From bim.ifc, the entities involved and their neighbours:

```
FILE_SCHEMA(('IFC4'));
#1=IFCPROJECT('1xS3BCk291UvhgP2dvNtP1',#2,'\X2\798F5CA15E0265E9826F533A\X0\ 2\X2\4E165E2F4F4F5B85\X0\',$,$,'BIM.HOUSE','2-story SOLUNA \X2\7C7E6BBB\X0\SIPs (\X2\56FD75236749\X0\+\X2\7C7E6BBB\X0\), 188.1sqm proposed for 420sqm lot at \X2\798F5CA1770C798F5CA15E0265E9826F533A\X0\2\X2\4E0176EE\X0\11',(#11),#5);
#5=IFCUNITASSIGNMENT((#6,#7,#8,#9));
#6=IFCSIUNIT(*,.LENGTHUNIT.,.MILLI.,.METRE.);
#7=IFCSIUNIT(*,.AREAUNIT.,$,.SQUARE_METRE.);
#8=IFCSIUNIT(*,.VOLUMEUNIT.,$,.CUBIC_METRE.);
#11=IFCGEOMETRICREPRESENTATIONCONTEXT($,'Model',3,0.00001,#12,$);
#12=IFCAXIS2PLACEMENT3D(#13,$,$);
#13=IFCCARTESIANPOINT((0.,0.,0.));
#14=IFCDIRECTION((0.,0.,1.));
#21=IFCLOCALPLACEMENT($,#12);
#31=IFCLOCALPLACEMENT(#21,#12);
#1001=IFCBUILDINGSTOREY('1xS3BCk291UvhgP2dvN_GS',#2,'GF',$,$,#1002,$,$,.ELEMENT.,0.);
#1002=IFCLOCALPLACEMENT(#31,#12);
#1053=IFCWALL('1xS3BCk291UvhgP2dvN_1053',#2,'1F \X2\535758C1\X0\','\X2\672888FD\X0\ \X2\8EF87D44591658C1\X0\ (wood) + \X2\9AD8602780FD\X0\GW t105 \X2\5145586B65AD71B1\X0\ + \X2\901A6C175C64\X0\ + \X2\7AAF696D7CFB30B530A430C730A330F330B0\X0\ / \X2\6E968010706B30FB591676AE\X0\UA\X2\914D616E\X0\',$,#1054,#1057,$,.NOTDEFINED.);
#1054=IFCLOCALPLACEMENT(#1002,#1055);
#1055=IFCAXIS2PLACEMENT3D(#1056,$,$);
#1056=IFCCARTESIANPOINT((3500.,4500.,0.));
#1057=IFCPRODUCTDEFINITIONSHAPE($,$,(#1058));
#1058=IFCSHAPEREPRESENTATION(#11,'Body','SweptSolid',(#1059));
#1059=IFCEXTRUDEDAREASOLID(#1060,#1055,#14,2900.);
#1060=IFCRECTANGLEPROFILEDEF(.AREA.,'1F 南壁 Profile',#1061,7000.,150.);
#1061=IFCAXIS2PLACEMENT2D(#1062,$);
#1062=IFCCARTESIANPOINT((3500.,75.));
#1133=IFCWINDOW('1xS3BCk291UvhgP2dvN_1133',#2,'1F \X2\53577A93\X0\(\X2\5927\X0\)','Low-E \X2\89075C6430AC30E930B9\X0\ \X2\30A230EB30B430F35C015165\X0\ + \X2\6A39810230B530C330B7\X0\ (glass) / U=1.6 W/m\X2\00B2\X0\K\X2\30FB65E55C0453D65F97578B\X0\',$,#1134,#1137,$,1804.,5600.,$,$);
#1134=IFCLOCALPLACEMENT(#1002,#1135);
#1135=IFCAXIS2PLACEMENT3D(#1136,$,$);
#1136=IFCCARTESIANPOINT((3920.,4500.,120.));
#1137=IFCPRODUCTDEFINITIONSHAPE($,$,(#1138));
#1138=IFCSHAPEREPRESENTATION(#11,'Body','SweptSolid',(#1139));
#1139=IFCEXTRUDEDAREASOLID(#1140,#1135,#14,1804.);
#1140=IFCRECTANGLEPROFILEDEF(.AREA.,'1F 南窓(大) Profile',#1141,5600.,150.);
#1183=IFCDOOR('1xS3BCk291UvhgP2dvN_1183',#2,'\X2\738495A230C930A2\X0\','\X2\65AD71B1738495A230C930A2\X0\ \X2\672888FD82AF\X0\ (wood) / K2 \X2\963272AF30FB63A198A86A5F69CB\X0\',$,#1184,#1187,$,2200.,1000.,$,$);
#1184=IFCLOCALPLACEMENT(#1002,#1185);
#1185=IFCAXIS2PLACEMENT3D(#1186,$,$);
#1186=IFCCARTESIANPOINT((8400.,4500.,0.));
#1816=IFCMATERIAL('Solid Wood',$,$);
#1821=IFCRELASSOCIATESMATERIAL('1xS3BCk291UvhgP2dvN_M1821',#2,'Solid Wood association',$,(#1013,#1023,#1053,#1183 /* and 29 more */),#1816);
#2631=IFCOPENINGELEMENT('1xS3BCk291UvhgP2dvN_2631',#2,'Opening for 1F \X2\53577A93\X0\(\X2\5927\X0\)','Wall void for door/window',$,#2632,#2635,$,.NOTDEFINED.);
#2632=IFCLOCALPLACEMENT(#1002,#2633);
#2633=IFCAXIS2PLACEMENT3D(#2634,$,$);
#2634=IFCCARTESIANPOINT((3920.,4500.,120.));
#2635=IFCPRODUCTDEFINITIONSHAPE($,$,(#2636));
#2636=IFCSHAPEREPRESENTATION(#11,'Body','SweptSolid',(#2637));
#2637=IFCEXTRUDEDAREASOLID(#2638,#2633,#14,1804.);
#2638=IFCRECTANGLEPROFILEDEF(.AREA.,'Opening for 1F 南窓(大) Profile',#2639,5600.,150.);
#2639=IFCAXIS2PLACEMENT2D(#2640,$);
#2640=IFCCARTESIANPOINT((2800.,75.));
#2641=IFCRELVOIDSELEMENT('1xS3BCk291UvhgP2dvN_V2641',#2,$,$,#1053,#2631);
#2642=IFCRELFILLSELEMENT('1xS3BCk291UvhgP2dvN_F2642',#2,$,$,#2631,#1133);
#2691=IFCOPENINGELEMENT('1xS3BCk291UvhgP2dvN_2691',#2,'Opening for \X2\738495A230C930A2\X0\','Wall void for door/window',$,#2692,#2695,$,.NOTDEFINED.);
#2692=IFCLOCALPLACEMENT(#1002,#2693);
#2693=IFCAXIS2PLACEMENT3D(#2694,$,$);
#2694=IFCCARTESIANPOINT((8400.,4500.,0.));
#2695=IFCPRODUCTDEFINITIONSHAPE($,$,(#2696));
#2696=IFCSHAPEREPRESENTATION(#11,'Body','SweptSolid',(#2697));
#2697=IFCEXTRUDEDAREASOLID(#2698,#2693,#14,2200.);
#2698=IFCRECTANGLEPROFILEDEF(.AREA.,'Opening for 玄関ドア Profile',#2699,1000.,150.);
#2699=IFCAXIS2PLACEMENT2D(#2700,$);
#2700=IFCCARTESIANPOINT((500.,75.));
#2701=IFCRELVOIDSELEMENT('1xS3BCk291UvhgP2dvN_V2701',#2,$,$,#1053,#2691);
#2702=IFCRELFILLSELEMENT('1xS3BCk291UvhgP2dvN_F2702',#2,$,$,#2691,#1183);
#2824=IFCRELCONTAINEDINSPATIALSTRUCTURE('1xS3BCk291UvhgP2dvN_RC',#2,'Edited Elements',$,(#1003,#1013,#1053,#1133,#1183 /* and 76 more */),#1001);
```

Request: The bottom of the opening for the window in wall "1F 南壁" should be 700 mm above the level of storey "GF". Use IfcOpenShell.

```python
import numpy as np
import ifcopenshell
import ifcopenshell.api.geometry
import ifcopenshell.geom
import ifcopenshell.util.element
import ifcopenshell.util.placement
import ifcopenshell.util.shape
import ifcopenshell.util.unit

model = ifcopenshell.open("bim.ifc")
unit_scale = ifcopenshell.util.unit.calculate_unit_scale(model)

window = model.by_guid("1xS3BCk291UvhgP2dvN_1133")
opening = window.FillsVoids[0].RelatingOpeningElement
storey = ifcopenshell.util.element.get_container(window, ifc_class="IfcBuildingStorey")
level = ifcopenshell.util.placement.get_local_placement(storey.ObjectPlacement)[2, 3]

# The opening's origin need not be at the sill, so measure its lowest point.
shape = ifcopenshell.geom.create_shape(ifcopenshell.geom.settings(), opening)
bottom = ifcopenshell.util.shape.get_shape_bottom_elevation(shape, shape.geometry) / unit_scale
dz = level + 0.7 / unit_scale - bottom

shift = np.array([0.0, 0.0, dz])
# The window is not placed relative to its opening, so move both.
for product in (opening, window):
    matrix = ifcopenshell.util.placement.get_local_placement(product.ObjectPlacement)
    matrix[:3, 3] += shift
    ifcopenshell.api.geometry.edit_object_placement(model, product=product, matrix=matrix, is_si=False)

print(f"moved by {dz * unit_scale:+.3f} m")

model.write("bim_edited.ifc")
```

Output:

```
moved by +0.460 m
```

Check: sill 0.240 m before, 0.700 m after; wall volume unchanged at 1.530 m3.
